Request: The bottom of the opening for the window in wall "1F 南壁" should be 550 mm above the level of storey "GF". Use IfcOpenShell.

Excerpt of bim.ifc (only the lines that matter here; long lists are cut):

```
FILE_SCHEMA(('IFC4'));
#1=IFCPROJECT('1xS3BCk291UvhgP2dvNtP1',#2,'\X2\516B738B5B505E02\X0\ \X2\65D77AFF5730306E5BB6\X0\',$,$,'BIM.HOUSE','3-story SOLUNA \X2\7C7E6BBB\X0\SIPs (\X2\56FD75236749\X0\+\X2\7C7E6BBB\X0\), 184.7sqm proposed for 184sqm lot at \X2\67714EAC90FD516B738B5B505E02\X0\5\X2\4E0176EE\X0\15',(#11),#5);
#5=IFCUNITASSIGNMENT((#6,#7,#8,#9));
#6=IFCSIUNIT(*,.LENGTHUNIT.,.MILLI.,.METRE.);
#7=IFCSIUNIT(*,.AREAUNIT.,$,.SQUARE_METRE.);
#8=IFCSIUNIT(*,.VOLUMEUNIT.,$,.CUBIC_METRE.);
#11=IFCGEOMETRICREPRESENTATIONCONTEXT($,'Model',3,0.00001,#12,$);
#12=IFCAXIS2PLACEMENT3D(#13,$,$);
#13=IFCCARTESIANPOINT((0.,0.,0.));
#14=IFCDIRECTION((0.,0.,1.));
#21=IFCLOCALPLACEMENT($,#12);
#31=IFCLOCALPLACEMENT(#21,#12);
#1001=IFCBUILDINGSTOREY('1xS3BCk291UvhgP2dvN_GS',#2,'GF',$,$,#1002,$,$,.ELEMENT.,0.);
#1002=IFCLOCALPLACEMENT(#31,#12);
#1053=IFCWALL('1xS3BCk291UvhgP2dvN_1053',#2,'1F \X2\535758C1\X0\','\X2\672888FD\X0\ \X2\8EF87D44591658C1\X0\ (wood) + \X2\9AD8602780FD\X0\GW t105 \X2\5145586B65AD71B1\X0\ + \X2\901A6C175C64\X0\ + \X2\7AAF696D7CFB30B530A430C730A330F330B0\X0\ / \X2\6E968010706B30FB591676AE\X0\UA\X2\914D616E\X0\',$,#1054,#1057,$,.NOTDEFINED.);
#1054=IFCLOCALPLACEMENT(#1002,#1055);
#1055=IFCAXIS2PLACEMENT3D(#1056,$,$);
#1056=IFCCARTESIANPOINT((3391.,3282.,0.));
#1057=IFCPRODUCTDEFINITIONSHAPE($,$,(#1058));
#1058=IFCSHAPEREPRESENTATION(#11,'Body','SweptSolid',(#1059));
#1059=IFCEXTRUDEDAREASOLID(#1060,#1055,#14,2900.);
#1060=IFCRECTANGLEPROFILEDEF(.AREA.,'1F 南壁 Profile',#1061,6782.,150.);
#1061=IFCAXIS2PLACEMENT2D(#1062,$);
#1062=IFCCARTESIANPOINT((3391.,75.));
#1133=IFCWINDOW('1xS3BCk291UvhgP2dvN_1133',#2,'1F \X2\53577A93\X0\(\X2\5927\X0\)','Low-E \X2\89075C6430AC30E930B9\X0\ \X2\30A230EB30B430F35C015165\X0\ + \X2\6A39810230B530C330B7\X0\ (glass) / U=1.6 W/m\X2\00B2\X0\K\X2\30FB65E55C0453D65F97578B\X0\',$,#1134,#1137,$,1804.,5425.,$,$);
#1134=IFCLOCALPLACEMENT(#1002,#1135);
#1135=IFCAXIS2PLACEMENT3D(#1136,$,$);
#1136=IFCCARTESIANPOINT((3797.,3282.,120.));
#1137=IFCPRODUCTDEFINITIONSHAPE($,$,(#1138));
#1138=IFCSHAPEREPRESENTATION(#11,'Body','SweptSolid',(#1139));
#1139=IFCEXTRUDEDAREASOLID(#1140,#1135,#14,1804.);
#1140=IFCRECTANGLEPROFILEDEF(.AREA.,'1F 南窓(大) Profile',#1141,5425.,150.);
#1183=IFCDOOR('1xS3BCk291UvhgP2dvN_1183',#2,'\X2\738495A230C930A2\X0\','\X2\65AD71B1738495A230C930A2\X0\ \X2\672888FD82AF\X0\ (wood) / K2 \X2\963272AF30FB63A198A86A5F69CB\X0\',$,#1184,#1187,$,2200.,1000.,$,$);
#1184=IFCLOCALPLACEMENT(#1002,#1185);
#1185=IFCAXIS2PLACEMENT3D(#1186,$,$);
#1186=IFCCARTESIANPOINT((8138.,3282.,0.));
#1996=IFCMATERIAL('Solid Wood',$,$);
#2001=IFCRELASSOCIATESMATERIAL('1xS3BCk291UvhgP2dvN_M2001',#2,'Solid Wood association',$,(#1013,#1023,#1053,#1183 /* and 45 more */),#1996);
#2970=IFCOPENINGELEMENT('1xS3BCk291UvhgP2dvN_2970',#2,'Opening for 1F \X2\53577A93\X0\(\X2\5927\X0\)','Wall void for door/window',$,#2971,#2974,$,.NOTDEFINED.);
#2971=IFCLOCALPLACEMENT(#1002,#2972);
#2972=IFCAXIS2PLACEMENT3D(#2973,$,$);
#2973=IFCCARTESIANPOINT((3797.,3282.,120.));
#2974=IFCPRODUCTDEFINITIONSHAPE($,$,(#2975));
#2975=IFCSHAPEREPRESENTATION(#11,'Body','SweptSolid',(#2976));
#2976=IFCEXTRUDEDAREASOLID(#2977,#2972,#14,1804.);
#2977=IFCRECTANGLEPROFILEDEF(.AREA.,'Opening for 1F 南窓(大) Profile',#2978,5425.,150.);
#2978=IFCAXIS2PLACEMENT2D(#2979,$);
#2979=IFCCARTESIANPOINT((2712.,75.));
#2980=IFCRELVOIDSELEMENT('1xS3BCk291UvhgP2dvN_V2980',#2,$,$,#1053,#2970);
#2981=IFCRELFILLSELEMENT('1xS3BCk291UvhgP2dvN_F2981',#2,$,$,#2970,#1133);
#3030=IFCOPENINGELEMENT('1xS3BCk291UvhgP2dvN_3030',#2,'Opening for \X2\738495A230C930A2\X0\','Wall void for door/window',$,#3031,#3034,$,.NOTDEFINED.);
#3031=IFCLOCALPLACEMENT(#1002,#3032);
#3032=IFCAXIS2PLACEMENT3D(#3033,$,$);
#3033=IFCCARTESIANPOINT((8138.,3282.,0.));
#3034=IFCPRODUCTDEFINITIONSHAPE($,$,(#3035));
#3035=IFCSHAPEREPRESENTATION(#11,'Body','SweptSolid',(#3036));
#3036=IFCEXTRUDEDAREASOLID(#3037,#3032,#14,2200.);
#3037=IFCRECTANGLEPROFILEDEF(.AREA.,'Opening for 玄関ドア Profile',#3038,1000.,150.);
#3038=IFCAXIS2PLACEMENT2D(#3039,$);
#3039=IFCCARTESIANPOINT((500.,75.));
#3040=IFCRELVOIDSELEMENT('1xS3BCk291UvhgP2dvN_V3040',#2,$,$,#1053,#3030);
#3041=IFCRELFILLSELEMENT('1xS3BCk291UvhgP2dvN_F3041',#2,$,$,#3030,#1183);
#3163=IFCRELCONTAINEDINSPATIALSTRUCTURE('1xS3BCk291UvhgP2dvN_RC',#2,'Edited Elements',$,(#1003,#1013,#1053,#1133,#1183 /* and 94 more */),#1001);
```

```python
import numpy as np
import ifcopenshell
import ifcopenshell.api.geometry
import ifcopenshell.geom
import ifcopenshell.util.element
import ifcopenshell.util.placement
import ifcopenshell.util.shape
import ifcopenshell.util.unit

model = ifcopenshell.open("bim.ifc")
unit_scale = ifcopenshell.util.unit.calculate_unit_scale(model)

window = model.by_guid("1xS3BCk291UvhgP2dvN_1133")
opening = window.FillsVoids[0].RelatingOpeningElement
storey = ifcopenshell.util.element.get_container(window, ifc_class="IfcBuildingStorey")
level = ifcopenshell.util.placement.get_local_placement(storey.ObjectPlacement)[2, 3]

# The opening's origin need not be at the sill, so measure its lowest point.
shape = ifcopenshell.geom.create_shape(ifcopenshell.geom.settings(), opening)
bottom = ifcopenshell.util.shape.get_shape_bottom_elevation(shape, shape.geometry) / unit_scale
dz = level + 0.55 / unit_scale - bottom

shift = np.array([0.0, 0.0, dz])
# The window is not placed relative to its opening, so move both.
for product in (opening, window):
    matrix = ifcopenshell.util.placement.get_local_placement(product.ObjectPlacement)
    matrix[:3, 3] += shift
    ifcopenshell.api.geometry.edit_object_placement(model, product=product, matrix=matrix, is_si=False)

print(f"moved by {dz * unit_scale:+.3f} m")

model.write("bim_rev.ifc")
```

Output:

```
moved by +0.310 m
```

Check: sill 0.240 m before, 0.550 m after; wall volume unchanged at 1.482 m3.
